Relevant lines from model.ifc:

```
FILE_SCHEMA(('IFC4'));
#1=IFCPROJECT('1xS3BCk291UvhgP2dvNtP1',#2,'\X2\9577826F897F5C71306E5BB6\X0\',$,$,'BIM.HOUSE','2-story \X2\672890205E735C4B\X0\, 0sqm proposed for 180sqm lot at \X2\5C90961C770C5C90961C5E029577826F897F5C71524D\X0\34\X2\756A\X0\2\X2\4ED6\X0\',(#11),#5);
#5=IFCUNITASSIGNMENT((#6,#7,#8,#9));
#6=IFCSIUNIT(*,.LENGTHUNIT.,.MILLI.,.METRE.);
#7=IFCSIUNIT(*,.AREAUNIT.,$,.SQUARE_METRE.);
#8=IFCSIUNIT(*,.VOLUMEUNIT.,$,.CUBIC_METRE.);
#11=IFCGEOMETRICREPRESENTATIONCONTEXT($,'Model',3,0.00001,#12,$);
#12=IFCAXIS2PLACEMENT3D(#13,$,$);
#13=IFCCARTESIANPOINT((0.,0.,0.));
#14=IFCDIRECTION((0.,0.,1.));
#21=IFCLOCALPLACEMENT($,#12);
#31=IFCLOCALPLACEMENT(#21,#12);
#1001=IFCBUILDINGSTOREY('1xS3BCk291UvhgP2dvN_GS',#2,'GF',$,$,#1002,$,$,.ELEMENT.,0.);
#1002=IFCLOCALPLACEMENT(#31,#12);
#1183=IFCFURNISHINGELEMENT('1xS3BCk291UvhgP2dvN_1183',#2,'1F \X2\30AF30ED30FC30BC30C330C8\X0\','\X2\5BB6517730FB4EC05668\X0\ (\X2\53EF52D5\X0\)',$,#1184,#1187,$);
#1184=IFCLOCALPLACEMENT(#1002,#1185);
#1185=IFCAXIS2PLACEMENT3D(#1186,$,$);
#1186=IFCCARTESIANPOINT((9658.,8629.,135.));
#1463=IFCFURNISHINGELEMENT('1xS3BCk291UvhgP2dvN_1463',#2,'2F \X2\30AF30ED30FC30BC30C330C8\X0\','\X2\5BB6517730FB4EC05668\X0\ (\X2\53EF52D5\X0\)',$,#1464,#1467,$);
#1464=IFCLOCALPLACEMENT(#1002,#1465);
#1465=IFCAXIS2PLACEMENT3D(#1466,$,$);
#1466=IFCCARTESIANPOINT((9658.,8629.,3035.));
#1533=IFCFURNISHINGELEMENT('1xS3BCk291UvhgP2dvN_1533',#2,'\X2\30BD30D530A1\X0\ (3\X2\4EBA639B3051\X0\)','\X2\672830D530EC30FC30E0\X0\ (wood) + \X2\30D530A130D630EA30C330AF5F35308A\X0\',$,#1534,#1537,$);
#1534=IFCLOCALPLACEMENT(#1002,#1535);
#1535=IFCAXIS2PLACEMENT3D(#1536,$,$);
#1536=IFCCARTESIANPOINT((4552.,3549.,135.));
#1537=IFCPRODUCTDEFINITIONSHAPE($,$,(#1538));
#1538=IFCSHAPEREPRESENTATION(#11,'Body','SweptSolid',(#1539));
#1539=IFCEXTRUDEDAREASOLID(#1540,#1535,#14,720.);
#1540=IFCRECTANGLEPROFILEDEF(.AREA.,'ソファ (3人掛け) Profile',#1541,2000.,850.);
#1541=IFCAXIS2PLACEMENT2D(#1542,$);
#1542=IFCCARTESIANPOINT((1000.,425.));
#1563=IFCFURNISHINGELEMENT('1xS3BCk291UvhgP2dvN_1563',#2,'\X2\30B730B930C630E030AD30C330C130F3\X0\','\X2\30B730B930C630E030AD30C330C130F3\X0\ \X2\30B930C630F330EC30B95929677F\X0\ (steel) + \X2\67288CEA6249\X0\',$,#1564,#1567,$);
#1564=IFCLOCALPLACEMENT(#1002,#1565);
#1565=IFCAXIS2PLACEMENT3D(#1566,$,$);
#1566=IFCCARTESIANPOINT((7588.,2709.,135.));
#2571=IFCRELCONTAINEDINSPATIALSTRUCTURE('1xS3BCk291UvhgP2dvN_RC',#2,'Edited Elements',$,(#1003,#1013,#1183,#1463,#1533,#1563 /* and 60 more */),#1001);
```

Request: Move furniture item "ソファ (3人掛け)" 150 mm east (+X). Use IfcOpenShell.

```python
import ifcopenshell
import ifcopenshell.api.geometry
import ifcopenshell.util.placement

model = ifcopenshell.open("model.ifc")

item = model.by_id(1533)
matrix = ifcopenshell.util.placement.get_local_placement(item.ObjectPlacement)
matrix[0, 3] += 150.0
ifcopenshell.api.geometry.edit_object_placement(model, product=item, matrix=matrix, is_si=False)

print(ifcopenshell.util.placement.get_local_placement(item.ObjectPlacement).round(3) + 0.0)

model.write("model-out.ifc")
```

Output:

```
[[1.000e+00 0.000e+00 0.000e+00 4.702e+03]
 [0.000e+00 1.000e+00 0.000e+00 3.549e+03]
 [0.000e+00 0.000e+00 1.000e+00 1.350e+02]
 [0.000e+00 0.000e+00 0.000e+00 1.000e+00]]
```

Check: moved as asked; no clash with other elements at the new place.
